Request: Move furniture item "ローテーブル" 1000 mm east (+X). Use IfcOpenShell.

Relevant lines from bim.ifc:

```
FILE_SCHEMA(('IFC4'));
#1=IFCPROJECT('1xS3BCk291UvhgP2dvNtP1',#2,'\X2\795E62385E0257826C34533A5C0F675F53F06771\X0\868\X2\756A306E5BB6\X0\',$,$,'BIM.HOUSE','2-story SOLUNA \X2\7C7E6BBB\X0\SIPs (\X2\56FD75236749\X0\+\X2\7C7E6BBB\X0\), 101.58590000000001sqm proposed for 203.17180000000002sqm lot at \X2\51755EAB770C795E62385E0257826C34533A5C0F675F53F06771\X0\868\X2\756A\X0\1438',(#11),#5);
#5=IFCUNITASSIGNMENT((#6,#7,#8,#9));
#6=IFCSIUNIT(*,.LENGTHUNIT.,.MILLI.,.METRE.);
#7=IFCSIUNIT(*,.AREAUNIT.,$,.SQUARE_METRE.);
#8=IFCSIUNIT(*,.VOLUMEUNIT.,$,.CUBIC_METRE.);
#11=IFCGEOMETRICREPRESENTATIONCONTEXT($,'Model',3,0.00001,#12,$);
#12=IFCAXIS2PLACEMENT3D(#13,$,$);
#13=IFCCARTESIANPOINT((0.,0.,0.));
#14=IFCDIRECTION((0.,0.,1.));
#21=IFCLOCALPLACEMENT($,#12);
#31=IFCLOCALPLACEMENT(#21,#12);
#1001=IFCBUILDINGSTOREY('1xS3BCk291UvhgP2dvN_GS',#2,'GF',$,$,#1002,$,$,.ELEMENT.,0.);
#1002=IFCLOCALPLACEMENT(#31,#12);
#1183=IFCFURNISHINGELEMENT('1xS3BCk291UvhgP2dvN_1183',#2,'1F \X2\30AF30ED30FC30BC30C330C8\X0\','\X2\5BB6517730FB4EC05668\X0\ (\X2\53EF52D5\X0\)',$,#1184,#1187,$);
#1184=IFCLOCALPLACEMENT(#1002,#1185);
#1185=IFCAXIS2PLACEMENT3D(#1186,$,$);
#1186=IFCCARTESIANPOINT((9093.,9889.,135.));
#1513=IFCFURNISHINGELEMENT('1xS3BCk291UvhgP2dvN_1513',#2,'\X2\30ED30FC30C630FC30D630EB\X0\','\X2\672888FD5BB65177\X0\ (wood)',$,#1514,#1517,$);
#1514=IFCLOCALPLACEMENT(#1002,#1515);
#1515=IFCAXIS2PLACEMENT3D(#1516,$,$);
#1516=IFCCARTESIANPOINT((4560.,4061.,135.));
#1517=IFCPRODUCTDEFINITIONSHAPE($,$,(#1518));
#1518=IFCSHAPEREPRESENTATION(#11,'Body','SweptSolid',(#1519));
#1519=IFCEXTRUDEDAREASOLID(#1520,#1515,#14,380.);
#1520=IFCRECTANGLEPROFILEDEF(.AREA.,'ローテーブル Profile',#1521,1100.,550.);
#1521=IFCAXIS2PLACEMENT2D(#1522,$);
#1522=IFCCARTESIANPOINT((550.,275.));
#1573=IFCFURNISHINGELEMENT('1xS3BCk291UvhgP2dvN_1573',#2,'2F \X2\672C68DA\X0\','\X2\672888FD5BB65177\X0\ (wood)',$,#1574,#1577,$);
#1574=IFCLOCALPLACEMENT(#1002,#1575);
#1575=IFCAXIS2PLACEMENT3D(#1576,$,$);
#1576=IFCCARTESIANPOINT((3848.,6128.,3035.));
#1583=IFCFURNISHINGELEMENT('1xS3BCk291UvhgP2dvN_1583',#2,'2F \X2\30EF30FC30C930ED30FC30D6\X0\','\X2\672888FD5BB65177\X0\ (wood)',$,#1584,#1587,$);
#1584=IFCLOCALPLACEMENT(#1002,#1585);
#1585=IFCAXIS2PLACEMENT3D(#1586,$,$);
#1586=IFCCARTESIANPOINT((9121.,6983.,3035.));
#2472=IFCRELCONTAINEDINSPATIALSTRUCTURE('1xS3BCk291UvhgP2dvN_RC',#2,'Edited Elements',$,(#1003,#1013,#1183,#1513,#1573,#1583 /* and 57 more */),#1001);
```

```python
import ifcopenshell
import ifcopenshell.api.geometry
import ifcopenshell.util.placement

model = ifcopenshell.open("bim.ifc")

item = model.by_guid("1xS3BCk291UvhgP2dvN_1513")
matrix = ifcopenshell.util.placement.get_local_placement(item.ObjectPlacement)
matrix[0, 3] += 1000.0
ifcopenshell.api.geometry.edit_object_placement(model, product=item, matrix=matrix, is_si=False)

print(ifcopenshell.util.placement.get_local_placement(item.ObjectPlacement).round(3) + 0.0)

model.write("bim-out.ifc")
```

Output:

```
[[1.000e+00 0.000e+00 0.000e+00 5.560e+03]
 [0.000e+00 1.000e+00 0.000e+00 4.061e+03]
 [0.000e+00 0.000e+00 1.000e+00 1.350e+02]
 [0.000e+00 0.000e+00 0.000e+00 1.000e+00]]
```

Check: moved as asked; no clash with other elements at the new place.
